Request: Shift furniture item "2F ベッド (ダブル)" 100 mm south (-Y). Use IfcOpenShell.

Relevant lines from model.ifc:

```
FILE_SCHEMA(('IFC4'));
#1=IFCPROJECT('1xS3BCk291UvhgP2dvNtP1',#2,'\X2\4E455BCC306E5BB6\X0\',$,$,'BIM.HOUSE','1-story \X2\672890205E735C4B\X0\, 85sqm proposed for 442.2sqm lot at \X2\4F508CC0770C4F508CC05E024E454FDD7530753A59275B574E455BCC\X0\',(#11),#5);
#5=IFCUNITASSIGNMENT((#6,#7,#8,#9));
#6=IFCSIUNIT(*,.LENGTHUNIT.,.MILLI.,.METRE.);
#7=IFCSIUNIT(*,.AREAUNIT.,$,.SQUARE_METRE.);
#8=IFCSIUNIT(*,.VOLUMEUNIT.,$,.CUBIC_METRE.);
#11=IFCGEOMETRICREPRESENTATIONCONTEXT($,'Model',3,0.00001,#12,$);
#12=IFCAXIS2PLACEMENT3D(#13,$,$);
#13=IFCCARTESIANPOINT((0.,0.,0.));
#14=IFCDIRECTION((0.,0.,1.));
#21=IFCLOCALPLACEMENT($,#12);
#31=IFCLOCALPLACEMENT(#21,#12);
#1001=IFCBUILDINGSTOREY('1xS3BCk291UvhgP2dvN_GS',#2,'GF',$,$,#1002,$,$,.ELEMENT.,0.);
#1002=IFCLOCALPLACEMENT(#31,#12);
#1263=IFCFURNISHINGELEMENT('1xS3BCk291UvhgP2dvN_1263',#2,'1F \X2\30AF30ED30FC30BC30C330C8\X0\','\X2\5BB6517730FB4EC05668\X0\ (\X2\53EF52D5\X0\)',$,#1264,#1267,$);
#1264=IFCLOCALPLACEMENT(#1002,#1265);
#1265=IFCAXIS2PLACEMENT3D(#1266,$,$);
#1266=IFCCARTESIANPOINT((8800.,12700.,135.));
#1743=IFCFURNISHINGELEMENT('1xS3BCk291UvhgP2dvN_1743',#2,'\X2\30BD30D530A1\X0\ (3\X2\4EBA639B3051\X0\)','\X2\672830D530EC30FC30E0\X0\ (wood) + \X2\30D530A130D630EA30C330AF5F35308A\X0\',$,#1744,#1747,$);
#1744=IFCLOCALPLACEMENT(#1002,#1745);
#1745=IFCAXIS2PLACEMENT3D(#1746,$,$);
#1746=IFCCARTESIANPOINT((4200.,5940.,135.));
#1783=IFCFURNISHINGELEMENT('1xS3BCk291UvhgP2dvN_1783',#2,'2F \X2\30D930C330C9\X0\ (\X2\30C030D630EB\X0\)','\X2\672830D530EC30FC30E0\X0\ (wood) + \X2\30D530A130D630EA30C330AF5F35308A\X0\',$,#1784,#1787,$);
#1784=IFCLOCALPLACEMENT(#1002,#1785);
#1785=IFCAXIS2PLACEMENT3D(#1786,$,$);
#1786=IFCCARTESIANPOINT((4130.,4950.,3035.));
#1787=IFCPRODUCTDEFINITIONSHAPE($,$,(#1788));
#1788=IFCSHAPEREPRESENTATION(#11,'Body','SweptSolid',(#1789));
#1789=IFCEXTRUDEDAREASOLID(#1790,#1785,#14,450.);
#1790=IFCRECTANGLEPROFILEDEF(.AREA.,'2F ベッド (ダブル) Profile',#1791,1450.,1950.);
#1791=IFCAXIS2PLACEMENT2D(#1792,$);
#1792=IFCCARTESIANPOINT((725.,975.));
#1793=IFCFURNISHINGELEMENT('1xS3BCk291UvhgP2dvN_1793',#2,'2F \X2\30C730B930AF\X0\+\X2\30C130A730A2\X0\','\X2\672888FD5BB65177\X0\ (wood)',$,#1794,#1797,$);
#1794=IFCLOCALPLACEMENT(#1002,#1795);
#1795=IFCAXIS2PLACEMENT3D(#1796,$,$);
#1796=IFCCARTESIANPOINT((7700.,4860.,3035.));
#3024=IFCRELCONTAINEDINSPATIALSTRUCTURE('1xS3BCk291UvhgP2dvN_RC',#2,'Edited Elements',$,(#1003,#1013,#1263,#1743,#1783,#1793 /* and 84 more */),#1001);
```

```python
import ifcopenshell
import ifcopenshell.api.geometry
import ifcopenshell.util.placement
import ifcopenshell.util.unit

model = ifcopenshell.open("model.ifc")
unit_scale = ifcopenshell.util.unit.calculate_unit_scale(model)

item = model.by_guid("1xS3BCk291UvhgP2dvN_1783")
matrix = ifcopenshell.util.placement.get_local_placement(item.ObjectPlacement)
matrix[1, 3] -= 0.1 / unit_scale
ifcopenshell.api.geometry.edit_object_placement(model, product=item, matrix=matrix, is_si=False)

print(ifcopenshell.util.placement.get_local_placement(item.ObjectPlacement).round(3) + 0.0)

model.write("model_rev.ifc")
```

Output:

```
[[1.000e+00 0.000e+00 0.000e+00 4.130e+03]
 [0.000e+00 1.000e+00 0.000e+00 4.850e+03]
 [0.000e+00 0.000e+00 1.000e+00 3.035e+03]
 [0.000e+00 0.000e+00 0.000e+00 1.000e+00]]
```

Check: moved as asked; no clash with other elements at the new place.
